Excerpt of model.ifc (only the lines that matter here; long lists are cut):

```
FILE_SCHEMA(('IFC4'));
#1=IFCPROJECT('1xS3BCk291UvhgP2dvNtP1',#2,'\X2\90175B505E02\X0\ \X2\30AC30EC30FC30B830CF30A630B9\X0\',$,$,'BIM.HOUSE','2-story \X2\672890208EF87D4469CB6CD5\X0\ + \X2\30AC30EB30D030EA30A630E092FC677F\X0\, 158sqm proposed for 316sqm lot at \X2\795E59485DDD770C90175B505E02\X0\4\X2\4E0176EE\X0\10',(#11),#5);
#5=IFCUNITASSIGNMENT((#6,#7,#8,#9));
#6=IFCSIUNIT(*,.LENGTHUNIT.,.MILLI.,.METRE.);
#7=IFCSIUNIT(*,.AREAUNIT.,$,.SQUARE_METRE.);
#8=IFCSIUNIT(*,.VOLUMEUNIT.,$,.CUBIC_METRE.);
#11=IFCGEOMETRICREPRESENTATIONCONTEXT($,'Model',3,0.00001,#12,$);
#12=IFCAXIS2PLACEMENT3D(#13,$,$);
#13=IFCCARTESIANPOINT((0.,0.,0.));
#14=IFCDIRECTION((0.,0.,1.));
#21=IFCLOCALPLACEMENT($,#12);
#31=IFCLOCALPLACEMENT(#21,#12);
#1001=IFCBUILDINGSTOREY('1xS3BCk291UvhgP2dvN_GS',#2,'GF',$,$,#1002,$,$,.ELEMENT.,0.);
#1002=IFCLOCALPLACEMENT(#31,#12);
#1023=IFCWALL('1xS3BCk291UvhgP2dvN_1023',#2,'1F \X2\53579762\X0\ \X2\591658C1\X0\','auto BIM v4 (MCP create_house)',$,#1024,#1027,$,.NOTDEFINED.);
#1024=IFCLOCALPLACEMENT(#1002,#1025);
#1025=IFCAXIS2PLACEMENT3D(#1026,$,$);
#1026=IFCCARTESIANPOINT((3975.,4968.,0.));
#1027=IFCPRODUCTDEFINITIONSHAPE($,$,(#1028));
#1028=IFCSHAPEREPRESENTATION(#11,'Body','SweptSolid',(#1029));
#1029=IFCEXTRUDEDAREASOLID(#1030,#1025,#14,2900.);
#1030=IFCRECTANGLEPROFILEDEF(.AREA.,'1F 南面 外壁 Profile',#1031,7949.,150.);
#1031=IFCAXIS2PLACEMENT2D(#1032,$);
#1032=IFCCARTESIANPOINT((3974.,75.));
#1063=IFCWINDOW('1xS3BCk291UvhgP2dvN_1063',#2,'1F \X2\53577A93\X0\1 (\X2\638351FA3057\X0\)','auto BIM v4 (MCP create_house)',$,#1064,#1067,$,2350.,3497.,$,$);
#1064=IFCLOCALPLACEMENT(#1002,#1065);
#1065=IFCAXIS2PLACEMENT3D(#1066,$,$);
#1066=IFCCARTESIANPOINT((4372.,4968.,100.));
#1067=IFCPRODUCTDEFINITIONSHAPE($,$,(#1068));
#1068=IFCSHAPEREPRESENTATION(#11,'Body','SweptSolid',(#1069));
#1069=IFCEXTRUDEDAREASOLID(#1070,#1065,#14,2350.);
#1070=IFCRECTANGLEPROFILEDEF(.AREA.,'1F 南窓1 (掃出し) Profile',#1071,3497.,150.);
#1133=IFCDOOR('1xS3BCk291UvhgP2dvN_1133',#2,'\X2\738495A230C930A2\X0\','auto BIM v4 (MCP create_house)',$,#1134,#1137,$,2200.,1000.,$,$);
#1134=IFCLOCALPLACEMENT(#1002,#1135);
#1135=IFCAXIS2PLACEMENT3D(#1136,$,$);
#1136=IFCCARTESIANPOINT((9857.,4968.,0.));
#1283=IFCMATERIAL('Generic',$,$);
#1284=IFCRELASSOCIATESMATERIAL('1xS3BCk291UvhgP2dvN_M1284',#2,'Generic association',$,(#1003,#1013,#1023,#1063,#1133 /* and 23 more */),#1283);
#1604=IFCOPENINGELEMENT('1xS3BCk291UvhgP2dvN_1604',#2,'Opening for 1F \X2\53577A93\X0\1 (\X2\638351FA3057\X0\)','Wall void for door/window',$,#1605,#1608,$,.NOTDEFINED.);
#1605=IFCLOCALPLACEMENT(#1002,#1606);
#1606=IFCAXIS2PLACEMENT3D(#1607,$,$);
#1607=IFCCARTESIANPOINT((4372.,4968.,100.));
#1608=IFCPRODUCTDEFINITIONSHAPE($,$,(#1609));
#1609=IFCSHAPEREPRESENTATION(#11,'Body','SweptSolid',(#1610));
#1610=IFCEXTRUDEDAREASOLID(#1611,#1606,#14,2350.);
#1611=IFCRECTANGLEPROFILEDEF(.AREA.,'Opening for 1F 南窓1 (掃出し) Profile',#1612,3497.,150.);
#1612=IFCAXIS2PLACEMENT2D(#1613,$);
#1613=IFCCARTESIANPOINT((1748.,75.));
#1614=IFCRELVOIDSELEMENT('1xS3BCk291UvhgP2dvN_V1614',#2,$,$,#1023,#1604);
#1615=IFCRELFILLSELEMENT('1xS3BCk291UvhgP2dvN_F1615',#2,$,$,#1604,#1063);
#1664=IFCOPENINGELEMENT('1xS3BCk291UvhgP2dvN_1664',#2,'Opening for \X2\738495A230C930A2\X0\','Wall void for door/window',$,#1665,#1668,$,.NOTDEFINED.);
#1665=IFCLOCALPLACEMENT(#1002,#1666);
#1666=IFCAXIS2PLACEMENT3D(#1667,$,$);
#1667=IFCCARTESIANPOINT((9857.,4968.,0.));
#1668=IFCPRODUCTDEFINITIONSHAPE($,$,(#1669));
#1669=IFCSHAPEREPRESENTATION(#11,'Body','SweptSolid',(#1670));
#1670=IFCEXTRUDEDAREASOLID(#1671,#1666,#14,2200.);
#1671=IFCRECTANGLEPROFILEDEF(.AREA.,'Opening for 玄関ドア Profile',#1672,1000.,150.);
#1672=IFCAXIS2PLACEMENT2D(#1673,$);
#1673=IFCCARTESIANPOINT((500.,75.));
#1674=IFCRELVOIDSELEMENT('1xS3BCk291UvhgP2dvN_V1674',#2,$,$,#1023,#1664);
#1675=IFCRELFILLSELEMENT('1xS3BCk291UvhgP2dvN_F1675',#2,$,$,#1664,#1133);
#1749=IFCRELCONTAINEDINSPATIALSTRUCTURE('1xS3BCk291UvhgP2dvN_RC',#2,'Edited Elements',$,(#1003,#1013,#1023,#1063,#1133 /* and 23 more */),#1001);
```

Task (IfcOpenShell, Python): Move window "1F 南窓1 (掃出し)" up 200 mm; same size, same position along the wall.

```python
import numpy as np
import ifcopenshell
import ifcopenshell.api.geometry
import ifcopenshell.util.placement
import ifcopenshell.util.unit

model = ifcopenshell.open("model.ifc")
unit_scale = ifcopenshell.util.unit.calculate_unit_scale(model)

window = model.by_guid("1xS3BCk291UvhgP2dvN_1063")
opening = window.FillsVoids[0].RelatingOpeningElement
dz = 0.2 / unit_scale

shift = np.array([0.0, 0.0, dz])
# The window is not placed relative to its opening, so move both.
for product in (opening, window):
    matrix = ifcopenshell.util.placement.get_local_placement(product.ObjectPlacement)
    matrix[:3, 3] += shift
    ifcopenshell.api.geometry.edit_object_placement(model, product=product, matrix=matrix, is_si=False)

print(f"moved by {dz * unit_scale:+.3f} m")

model.write("model_updated.ifc")
```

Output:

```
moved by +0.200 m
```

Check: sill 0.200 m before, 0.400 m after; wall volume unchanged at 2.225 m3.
